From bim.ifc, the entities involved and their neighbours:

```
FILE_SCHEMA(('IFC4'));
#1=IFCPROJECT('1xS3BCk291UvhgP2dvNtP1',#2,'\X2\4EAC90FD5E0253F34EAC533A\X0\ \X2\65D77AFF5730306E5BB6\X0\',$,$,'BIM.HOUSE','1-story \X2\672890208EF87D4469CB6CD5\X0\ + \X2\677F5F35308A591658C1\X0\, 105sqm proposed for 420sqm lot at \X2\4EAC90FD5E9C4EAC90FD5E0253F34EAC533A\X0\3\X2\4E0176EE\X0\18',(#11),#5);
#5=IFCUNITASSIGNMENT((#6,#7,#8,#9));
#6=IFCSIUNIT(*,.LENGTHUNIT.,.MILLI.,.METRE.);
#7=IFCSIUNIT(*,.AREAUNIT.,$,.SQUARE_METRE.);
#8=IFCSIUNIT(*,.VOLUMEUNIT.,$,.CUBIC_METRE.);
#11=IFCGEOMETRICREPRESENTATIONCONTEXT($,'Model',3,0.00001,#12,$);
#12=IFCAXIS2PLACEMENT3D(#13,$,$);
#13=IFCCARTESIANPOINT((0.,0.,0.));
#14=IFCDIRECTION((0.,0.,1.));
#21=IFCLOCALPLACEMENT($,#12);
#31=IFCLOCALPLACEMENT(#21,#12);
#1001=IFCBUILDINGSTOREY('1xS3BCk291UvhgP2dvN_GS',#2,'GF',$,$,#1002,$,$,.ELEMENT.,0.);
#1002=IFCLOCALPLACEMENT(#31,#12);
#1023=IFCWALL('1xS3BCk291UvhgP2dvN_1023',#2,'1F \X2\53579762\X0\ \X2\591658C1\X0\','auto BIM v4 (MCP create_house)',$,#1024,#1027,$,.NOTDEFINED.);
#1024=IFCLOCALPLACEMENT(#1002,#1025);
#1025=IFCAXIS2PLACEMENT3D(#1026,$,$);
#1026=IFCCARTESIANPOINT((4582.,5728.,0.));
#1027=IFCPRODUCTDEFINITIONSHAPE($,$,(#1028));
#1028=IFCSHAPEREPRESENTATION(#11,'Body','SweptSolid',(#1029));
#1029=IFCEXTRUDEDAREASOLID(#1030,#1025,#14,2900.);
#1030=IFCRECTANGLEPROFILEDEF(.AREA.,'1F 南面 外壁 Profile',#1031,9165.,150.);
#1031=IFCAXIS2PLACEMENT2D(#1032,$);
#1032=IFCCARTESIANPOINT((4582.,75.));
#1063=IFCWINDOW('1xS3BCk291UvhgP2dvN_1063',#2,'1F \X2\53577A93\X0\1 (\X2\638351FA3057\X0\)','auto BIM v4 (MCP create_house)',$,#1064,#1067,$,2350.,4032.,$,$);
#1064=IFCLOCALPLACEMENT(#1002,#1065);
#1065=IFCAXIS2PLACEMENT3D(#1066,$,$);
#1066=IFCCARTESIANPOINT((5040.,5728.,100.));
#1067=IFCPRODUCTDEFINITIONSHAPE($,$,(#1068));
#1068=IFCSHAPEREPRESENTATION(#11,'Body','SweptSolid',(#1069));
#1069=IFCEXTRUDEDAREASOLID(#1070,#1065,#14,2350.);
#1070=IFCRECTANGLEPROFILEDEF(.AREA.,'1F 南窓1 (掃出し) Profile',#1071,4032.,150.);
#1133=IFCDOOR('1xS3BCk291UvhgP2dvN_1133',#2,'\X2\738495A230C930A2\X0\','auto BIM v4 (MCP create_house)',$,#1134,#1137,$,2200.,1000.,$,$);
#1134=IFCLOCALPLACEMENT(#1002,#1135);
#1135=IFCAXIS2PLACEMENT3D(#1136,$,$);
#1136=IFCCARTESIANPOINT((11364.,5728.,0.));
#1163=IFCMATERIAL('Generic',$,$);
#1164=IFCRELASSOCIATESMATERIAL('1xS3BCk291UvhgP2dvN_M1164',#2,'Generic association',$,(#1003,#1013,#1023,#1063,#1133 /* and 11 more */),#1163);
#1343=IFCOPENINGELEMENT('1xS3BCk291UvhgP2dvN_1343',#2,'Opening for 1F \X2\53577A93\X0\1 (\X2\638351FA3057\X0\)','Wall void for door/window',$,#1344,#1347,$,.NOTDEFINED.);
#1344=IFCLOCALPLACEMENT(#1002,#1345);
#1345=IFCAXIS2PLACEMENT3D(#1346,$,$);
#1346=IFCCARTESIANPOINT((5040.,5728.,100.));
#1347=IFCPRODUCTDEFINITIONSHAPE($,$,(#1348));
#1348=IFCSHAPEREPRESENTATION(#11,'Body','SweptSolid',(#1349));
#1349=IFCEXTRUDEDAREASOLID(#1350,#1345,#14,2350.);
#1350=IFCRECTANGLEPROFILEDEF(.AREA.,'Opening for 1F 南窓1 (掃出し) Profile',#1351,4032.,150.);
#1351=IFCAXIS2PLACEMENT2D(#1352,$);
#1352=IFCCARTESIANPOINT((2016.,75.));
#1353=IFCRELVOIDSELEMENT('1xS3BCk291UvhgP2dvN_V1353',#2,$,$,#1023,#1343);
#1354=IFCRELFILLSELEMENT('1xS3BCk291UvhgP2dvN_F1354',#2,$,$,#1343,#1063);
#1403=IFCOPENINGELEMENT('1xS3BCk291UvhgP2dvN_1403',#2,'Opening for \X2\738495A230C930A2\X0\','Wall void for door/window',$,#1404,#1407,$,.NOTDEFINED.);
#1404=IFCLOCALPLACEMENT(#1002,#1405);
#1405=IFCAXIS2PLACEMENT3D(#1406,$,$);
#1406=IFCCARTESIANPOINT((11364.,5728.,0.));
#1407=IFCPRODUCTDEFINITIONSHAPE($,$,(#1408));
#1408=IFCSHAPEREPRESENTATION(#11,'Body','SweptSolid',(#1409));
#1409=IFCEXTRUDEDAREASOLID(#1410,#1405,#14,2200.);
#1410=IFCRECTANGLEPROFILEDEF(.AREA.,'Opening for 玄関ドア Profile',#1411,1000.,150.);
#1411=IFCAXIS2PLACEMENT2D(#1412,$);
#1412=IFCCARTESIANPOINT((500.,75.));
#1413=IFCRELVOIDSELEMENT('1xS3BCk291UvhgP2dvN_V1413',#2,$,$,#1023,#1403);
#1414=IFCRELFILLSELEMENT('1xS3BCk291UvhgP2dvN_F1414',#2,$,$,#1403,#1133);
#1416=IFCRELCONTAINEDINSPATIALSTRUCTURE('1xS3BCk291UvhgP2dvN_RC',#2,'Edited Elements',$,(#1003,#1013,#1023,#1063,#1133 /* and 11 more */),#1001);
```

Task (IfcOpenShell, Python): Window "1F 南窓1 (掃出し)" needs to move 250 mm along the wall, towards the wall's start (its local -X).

```python
import ifcopenshell
import ifcopenshell.api.geometry
import ifcopenshell.util.placement

model = ifcopenshell.open("bim.ifc")

window = model.by_id(1063)
opening = window.FillsVoids[0].RelatingOpeningElement
wall = opening.VoidsElements[0].RelatingBuildingElement

wall_matrix = ifcopenshell.util.placement.get_local_placement(wall.ObjectPlacement)
shift = wall_matrix[:3, 0] * -250.0
before = ifcopenshell.util.placement.get_local_placement(window.ObjectPlacement)[:3, 3].copy()

# The window is not placed relative to its opening, so move both.
for product in (opening, window):
    matrix = ifcopenshell.util.placement.get_local_placement(product.ObjectPlacement)
    matrix[:3, 3] += shift
    ifcopenshell.api.geometry.edit_object_placement(model, product=product, matrix=matrix, is_si=False)

after = ifcopenshell.util.placement.get_local_placement(window.ObjectPlacement)[:3, 3]
print("window moved by", (after - before).round(3) + 0.0)

model.write("bim_rev.ifc")
```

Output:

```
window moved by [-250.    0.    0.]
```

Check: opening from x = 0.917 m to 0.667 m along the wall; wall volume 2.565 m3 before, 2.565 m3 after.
